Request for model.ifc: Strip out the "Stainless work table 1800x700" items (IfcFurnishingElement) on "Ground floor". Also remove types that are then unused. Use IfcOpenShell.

First a look at what the model holds.

```python
import ifcopenshell
import ifcopenshell.util.element

model = ifcopenshell.open("model.ifc")
print(model.schema)
storey = next(s for s in model.by_type("IfcBuildingStorey") if s.Name == "Ground floor")
furniture = [e for e in ifcopenshell.util.element.get_decomposition(storey) if e.is_a("IfcFurnishingElement")]
seen = {}
for e in furniture:
    element_type = ifcopenshell.util.element.get_type(e)
    name = element_type.Name if element_type not in (None, e) else None
    seen[name] = seen.get(name, 0) + 1
for name, count in sorted(seen.items(), key=str):
    print(count, "x", name)
```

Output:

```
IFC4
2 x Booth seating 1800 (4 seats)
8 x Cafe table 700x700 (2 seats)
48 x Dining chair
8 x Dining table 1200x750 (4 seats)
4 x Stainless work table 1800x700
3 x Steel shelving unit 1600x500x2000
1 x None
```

```python
import ifcopenshell
import ifcopenshell.api.root
import ifcopenshell.util.element

model = ifcopenshell.open("model.ifc")

storey = next(s for s in model.by_type("IfcBuildingStorey") if s.Name == "Ground floor")
furniture = [e for e in ifcopenshell.util.element.get_decomposition(storey) if e.is_a("IfcFurnishingElement")]
targets = [e for e in furniture if (t := ifcopenshell.util.element.get_type(e)) not in (None, e) and t.Name == "Stainless work table 1800x700"]
types = {ifcopenshell.util.element.get_type(e) for e in targets} - {None, *targets}

for e in targets:
    ifcopenshell.api.root.remove_product(model, product=e)
print(len(targets), "removed")

unused = [t for t in types if not ifcopenshell.util.element.get_types(t)]
for t in unused:
    ifcopenshell.api.root.remove_product(model, product=t)
print(len(unused), "unused types removed")

model.write("model-out.ifc")
```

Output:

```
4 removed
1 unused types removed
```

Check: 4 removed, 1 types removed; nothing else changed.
